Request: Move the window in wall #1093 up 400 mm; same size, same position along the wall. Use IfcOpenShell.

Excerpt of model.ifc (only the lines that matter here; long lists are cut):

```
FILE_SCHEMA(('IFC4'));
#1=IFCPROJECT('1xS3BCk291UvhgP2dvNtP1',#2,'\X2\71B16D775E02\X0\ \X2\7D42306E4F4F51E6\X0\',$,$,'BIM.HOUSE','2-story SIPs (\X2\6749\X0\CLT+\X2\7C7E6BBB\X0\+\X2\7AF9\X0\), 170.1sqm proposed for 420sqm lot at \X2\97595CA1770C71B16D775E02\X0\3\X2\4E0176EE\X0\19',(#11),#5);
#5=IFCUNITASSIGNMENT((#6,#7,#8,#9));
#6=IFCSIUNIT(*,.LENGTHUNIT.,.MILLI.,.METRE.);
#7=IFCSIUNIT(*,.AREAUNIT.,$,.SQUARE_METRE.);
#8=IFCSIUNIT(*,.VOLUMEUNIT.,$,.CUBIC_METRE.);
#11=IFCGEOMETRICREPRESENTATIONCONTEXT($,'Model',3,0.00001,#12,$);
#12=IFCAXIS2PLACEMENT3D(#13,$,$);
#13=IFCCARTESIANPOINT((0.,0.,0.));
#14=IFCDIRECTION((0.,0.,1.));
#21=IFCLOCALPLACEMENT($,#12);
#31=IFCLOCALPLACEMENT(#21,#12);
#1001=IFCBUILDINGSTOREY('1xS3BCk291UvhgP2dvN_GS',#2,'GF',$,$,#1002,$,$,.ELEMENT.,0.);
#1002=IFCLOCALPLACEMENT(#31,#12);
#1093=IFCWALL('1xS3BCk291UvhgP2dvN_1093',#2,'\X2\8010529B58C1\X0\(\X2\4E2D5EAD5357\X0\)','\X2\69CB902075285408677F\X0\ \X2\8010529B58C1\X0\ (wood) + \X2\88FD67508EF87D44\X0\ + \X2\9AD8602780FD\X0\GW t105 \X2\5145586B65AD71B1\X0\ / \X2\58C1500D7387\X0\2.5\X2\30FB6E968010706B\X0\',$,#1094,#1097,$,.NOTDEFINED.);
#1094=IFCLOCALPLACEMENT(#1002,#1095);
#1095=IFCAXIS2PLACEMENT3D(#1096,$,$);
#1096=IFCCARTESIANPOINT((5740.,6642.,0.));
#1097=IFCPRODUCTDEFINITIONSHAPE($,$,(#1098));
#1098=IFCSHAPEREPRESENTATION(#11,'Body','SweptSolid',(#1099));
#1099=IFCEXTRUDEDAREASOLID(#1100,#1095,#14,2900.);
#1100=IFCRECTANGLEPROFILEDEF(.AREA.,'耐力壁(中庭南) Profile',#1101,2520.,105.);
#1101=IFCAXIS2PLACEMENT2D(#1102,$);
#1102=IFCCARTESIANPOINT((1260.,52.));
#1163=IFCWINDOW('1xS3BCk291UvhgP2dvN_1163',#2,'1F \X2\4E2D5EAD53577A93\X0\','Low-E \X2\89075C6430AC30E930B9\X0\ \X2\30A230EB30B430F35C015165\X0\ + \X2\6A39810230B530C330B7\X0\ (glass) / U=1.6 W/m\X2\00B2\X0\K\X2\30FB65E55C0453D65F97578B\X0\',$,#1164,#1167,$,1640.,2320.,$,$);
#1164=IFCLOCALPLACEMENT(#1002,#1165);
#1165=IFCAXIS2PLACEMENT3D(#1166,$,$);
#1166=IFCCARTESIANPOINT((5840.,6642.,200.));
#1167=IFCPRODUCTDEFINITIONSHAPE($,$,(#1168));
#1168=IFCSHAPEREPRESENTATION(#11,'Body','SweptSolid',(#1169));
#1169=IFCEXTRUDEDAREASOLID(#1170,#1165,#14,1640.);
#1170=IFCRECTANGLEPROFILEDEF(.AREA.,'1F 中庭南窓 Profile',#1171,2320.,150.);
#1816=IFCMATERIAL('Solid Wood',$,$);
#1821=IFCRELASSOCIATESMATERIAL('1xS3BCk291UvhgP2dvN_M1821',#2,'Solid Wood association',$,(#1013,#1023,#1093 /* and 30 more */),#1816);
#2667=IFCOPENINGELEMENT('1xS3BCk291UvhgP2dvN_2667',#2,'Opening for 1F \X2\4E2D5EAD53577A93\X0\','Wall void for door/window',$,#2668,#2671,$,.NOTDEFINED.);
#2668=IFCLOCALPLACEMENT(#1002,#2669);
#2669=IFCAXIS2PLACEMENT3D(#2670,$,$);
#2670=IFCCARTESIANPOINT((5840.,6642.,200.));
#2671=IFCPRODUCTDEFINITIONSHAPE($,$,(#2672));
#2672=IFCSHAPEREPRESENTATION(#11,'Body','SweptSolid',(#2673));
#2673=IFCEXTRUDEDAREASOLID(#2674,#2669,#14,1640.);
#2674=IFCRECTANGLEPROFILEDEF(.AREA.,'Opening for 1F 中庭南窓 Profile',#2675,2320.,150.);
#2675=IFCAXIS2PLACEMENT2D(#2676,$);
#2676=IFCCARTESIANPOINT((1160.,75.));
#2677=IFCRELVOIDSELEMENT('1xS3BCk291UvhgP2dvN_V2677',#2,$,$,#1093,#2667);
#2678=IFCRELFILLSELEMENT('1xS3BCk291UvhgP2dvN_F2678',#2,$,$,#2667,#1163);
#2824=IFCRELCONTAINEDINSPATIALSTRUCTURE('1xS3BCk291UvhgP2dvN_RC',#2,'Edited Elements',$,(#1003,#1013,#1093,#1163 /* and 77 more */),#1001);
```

```python
import numpy as np
import ifcopenshell
import ifcopenshell.api.geometry
import ifcopenshell.util.placement
import ifcopenshell.util.unit

model = ifcopenshell.open("model.ifc")
unit_scale = ifcopenshell.util.unit.calculate_unit_scale(model)

window = model.by_id(1163)
opening = window.FillsVoids[0].RelatingOpeningElement
dz = 0.4 / unit_scale

shift = np.array([0.0, 0.0, dz])
# The window is not placed relative to its opening, so move both.
for product in (opening, window):
    matrix = ifcopenshell.util.placement.get_local_placement(product.ObjectPlacement)
    matrix[:3, 3] += shift
    ifcopenshell.api.geometry.edit_object_placement(model, product=product, matrix=matrix, is_si=False)

print(f"moved by {dz * unit_scale:+.3f} m")

model.write("model-out.ifc")
```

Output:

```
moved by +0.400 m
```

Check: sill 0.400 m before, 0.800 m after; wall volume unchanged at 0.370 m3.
